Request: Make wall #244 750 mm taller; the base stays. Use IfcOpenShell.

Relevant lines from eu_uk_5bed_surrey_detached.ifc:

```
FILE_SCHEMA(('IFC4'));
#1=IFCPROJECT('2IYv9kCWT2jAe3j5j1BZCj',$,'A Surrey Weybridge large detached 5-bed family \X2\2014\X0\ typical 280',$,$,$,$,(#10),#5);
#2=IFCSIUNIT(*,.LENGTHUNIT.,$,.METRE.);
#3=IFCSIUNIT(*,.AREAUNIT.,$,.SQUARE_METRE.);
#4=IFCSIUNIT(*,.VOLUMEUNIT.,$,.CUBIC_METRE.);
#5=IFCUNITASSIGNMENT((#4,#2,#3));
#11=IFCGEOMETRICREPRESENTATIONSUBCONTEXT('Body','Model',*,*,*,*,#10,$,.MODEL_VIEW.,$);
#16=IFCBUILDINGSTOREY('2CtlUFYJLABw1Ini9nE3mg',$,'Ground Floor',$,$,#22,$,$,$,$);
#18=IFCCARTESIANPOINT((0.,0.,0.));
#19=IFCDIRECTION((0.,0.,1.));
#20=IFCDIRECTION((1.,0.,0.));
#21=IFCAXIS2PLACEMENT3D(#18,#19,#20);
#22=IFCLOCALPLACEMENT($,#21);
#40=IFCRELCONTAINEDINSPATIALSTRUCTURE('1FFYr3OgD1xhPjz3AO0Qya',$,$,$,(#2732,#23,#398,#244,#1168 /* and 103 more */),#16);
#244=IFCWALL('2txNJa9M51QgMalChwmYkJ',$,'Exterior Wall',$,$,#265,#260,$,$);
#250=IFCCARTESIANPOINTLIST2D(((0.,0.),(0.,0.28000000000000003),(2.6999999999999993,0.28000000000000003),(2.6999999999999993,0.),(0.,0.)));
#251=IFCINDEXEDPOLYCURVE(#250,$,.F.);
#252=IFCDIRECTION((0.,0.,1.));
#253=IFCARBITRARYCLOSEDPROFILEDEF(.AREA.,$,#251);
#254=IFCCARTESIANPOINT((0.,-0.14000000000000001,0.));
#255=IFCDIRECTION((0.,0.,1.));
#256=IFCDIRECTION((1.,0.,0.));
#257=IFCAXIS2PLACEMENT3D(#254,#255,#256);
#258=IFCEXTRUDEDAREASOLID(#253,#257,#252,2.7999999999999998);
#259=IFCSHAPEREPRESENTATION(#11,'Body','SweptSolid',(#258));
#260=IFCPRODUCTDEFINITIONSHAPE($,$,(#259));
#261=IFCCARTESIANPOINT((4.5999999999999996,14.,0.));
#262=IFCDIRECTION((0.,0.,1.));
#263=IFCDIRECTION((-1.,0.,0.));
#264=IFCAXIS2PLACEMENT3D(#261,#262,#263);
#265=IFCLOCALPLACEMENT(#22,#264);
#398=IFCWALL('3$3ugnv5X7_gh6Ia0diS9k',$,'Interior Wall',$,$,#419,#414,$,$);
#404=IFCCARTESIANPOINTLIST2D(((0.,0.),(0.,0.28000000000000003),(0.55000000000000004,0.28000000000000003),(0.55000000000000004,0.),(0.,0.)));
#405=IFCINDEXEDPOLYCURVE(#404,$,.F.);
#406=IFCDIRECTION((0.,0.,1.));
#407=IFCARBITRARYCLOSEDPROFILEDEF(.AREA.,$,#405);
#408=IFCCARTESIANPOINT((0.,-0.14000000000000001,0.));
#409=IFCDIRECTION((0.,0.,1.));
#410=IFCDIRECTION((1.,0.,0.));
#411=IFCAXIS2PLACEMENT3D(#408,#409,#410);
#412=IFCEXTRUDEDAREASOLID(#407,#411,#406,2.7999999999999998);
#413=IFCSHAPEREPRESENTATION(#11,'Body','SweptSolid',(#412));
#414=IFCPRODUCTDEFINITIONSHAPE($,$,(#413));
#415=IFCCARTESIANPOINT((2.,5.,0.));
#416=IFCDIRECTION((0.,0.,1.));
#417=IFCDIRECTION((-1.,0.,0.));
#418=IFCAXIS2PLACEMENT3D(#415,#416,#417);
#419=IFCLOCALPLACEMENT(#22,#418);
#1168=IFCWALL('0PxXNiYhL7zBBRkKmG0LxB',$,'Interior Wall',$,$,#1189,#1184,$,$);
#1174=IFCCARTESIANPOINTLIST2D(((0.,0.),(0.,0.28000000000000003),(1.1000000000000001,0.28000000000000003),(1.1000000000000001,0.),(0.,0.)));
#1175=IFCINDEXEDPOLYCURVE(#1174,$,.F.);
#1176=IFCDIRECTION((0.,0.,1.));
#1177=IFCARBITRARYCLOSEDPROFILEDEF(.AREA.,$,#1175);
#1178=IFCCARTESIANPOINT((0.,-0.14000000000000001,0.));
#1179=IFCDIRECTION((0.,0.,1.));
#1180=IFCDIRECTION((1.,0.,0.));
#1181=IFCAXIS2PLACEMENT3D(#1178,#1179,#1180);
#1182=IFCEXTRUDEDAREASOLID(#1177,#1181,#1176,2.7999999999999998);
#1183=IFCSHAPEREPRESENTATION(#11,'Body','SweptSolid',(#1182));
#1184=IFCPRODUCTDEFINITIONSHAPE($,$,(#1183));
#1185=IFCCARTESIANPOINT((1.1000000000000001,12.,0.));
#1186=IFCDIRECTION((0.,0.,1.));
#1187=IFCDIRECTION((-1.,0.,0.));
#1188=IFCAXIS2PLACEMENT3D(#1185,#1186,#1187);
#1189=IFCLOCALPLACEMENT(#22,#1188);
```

```python
import ifcopenshell
import ifcopenshell.geom
import ifcopenshell.util.representation
import ifcopenshell.util.shape
import ifcopenshell.util.unit

model = ifcopenshell.open("eu_uk_5bed_surrey_detached.ifc")
unit_scale = ifcopenshell.util.unit.calculate_unit_scale(model)
settings = ifcopenshell.geom.settings()


def volume(element):
    """Net volume in cubic metres, openings subtracted."""
    shape = ifcopenshell.geom.create_shape(settings, element)
    return ifcopenshell.util.shape.get_volume(shape.geometry)


wall = model.by_id(244)
before = volume(wall)

body = ifcopenshell.util.representation.get_representation(wall, "Model", "Body")
solid = body.Items[0]
old_height = solid.Depth
solid.Depth += 0.75 / unit_scale
after = volume(wall)

print(f"height {old_height:g} -> {solid.Depth:g}, volume {before:.3f} -> {after:.3f} m3")

model.write("eu_uk_5bed_surrey_detached_edited.ifc")
```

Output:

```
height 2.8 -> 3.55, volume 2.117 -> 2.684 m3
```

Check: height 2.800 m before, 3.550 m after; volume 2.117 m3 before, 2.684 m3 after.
